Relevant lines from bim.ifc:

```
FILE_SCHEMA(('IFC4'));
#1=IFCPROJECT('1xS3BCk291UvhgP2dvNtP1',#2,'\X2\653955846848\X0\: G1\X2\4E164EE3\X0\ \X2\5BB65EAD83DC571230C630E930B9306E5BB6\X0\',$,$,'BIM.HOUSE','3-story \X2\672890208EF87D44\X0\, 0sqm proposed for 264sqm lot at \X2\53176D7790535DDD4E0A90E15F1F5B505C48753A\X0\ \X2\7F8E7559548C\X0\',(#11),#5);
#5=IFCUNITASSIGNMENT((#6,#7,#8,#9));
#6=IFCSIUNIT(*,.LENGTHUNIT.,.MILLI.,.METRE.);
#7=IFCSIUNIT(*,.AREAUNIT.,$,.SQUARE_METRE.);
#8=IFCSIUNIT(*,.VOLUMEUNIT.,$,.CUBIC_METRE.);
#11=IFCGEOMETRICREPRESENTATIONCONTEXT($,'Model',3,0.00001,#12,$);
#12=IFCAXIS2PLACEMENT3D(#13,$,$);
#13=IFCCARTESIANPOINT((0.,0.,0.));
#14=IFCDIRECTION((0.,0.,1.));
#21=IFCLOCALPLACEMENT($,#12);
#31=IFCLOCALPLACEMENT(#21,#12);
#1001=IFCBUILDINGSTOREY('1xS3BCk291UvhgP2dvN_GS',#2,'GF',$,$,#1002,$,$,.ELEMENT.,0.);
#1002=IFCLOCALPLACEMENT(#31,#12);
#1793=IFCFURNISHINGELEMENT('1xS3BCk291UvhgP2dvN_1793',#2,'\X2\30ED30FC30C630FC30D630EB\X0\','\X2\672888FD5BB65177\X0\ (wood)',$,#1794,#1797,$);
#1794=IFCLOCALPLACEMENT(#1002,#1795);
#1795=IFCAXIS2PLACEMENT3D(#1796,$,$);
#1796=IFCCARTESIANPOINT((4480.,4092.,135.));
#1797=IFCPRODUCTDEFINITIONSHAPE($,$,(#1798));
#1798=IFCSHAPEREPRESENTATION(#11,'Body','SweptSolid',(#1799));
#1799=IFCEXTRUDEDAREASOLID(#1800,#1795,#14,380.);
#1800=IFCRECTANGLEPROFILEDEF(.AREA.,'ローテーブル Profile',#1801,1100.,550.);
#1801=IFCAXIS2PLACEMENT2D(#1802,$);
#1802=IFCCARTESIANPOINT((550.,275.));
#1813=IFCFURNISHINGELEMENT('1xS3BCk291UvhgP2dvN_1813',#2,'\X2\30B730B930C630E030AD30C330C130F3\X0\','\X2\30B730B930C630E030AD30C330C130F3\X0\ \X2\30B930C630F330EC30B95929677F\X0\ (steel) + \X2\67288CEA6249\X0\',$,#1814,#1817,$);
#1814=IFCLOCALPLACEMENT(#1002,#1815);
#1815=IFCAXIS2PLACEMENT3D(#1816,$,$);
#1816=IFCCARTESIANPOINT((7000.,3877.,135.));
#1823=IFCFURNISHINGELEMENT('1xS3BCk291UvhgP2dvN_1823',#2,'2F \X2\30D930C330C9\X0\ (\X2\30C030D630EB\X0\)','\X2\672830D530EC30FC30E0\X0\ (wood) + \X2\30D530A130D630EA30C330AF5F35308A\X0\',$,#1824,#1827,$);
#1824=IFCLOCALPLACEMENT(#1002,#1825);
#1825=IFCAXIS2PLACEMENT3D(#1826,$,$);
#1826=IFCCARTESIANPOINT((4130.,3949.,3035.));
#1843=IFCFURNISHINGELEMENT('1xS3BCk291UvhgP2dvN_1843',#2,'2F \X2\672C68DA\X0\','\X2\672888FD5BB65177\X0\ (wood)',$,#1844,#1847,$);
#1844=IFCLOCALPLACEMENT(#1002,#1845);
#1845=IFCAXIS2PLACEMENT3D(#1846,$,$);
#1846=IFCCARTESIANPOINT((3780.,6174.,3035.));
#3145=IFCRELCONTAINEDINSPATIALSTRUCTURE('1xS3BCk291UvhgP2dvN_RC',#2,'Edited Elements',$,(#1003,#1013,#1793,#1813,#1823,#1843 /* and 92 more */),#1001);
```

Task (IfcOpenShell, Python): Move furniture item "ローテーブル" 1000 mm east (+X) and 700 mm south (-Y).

```python
import ifcopenshell
import ifcopenshell.api.geometry
import ifcopenshell.util.placement

model = ifcopenshell.open("bim.ifc")

item = model.by_guid("1xS3BCk291UvhgP2dvN_1793")
matrix = ifcopenshell.util.placement.get_local_placement(item.ObjectPlacement)
matrix[0, 3] += 1000.0
matrix[1, 3] -= 700.0
ifcopenshell.api.geometry.edit_object_placement(model, product=item, matrix=matrix, is_si=False)

print(ifcopenshell.util.placement.get_local_placement(item.ObjectPlacement).round(3) + 0.0)

model.write("bim_v2.ifc")
```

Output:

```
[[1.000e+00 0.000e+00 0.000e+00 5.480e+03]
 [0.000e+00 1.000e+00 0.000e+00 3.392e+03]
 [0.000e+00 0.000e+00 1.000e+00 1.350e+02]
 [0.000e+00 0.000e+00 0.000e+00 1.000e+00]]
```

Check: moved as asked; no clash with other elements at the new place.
